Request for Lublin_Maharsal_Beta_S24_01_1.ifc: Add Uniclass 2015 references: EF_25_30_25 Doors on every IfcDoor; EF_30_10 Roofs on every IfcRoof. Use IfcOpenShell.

First a look at what the model holds.

```python
import ifcopenshell

model = ifcopenshell.open("Lublin_Maharsal_Beta_S24_01_1.ifc")
print(model.schema)
print("classifications:", [c.Name for c in model.by_type("IfcClassification")])
for ifc_class in ("IfcDoor", "IfcRoof", "IfcStair", "IfcWall", "IfcWindow"):
    print(ifc_class, len(model.by_type(ifc_class)))
```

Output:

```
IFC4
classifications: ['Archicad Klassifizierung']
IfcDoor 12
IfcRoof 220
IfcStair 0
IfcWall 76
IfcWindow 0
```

```python
import ifcopenshell
import ifcopenshell.api.classification

model = ifcopenshell.open("Lublin_Maharsal_Beta_S24_01_1.ifc")

system = ifcopenshell.api.classification.add_classification(model, classification="Uniclass 2015")

codes = {
    "IfcDoor": ("EF_25_30_25", "Doors"),
    "IfcRoof": ("EF_30_10", "Roofs"),
}
for ifc_class, (code, name) in codes.items():
    products = model.by_type(ifc_class)
    ifcopenshell.api.classification.add_reference(
        model, products=products, classification=system, identification=code, name=name
    )
    print(code, len(products))

model.write("Lublin_Maharsal_Beta_S24_01_1_rev.ifc")
```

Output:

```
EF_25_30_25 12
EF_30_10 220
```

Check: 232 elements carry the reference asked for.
